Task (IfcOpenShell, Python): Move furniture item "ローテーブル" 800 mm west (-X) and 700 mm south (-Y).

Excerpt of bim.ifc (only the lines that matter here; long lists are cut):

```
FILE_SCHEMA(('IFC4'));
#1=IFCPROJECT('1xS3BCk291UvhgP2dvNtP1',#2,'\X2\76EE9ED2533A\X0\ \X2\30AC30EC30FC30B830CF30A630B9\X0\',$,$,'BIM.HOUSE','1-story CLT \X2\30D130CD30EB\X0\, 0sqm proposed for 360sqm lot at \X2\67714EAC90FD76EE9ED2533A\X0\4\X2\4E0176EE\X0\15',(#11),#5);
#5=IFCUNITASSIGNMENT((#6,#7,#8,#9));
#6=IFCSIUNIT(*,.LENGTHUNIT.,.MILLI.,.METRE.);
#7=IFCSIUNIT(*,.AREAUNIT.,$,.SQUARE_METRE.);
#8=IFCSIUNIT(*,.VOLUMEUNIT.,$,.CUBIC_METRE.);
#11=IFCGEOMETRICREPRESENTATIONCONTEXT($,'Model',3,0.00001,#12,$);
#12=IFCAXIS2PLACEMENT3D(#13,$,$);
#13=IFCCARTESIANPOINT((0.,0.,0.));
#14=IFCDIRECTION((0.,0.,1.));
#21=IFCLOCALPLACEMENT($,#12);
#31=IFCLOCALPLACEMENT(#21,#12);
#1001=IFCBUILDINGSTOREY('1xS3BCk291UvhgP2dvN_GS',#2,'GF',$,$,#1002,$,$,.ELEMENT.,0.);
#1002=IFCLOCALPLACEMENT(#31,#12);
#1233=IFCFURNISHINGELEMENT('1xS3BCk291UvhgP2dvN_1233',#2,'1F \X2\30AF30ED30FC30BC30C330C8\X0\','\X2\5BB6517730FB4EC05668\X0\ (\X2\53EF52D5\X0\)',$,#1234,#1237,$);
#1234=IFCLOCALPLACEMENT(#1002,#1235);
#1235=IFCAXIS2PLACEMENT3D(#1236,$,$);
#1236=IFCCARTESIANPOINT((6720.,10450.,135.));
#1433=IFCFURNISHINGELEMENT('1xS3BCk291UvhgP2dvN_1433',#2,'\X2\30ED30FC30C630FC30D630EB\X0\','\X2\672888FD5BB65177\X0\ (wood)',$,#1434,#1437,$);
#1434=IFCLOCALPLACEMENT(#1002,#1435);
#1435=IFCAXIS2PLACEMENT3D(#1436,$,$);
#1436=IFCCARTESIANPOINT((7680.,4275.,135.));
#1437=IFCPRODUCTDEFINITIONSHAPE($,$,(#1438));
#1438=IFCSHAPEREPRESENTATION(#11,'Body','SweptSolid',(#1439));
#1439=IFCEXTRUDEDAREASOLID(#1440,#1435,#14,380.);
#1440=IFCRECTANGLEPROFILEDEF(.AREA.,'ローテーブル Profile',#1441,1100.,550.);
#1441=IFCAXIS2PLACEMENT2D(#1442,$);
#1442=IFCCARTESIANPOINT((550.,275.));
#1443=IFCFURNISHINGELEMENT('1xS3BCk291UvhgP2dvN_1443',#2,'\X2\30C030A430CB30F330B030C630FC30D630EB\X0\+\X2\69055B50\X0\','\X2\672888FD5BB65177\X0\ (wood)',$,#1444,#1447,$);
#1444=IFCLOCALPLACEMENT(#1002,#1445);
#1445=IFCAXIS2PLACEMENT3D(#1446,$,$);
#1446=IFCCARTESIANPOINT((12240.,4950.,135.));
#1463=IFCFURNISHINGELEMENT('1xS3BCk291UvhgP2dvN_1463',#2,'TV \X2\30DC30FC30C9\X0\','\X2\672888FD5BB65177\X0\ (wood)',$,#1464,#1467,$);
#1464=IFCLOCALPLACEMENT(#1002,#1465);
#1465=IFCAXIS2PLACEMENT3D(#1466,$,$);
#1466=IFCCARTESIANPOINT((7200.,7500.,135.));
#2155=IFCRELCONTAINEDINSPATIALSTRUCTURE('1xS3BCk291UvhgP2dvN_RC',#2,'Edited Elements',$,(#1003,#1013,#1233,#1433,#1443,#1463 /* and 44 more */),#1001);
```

```python
import ifcopenshell
import ifcopenshell.api.geometry
import ifcopenshell.util.placement
import ifcopenshell.util.unit

model = ifcopenshell.open("bim.ifc")
unit_scale = ifcopenshell.util.unit.calculate_unit_scale(model)

item = model.by_guid("1xS3BCk291UvhgP2dvN_1433")
matrix = ifcopenshell.util.placement.get_local_placement(item.ObjectPlacement)
matrix[0, 3] -= 0.8 / unit_scale
matrix[1, 3] -= 0.7 / unit_scale
ifcopenshell.api.geometry.edit_object_placement(model, product=item, matrix=matrix, is_si=False)

print(ifcopenshell.util.placement.get_local_placement(item.ObjectPlacement).round(3) + 0.0)

model.write("bim_edited.ifc")
```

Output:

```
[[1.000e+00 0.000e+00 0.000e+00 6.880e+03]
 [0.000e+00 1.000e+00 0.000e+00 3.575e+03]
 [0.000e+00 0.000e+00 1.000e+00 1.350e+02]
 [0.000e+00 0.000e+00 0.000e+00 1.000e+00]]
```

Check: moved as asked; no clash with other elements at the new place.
